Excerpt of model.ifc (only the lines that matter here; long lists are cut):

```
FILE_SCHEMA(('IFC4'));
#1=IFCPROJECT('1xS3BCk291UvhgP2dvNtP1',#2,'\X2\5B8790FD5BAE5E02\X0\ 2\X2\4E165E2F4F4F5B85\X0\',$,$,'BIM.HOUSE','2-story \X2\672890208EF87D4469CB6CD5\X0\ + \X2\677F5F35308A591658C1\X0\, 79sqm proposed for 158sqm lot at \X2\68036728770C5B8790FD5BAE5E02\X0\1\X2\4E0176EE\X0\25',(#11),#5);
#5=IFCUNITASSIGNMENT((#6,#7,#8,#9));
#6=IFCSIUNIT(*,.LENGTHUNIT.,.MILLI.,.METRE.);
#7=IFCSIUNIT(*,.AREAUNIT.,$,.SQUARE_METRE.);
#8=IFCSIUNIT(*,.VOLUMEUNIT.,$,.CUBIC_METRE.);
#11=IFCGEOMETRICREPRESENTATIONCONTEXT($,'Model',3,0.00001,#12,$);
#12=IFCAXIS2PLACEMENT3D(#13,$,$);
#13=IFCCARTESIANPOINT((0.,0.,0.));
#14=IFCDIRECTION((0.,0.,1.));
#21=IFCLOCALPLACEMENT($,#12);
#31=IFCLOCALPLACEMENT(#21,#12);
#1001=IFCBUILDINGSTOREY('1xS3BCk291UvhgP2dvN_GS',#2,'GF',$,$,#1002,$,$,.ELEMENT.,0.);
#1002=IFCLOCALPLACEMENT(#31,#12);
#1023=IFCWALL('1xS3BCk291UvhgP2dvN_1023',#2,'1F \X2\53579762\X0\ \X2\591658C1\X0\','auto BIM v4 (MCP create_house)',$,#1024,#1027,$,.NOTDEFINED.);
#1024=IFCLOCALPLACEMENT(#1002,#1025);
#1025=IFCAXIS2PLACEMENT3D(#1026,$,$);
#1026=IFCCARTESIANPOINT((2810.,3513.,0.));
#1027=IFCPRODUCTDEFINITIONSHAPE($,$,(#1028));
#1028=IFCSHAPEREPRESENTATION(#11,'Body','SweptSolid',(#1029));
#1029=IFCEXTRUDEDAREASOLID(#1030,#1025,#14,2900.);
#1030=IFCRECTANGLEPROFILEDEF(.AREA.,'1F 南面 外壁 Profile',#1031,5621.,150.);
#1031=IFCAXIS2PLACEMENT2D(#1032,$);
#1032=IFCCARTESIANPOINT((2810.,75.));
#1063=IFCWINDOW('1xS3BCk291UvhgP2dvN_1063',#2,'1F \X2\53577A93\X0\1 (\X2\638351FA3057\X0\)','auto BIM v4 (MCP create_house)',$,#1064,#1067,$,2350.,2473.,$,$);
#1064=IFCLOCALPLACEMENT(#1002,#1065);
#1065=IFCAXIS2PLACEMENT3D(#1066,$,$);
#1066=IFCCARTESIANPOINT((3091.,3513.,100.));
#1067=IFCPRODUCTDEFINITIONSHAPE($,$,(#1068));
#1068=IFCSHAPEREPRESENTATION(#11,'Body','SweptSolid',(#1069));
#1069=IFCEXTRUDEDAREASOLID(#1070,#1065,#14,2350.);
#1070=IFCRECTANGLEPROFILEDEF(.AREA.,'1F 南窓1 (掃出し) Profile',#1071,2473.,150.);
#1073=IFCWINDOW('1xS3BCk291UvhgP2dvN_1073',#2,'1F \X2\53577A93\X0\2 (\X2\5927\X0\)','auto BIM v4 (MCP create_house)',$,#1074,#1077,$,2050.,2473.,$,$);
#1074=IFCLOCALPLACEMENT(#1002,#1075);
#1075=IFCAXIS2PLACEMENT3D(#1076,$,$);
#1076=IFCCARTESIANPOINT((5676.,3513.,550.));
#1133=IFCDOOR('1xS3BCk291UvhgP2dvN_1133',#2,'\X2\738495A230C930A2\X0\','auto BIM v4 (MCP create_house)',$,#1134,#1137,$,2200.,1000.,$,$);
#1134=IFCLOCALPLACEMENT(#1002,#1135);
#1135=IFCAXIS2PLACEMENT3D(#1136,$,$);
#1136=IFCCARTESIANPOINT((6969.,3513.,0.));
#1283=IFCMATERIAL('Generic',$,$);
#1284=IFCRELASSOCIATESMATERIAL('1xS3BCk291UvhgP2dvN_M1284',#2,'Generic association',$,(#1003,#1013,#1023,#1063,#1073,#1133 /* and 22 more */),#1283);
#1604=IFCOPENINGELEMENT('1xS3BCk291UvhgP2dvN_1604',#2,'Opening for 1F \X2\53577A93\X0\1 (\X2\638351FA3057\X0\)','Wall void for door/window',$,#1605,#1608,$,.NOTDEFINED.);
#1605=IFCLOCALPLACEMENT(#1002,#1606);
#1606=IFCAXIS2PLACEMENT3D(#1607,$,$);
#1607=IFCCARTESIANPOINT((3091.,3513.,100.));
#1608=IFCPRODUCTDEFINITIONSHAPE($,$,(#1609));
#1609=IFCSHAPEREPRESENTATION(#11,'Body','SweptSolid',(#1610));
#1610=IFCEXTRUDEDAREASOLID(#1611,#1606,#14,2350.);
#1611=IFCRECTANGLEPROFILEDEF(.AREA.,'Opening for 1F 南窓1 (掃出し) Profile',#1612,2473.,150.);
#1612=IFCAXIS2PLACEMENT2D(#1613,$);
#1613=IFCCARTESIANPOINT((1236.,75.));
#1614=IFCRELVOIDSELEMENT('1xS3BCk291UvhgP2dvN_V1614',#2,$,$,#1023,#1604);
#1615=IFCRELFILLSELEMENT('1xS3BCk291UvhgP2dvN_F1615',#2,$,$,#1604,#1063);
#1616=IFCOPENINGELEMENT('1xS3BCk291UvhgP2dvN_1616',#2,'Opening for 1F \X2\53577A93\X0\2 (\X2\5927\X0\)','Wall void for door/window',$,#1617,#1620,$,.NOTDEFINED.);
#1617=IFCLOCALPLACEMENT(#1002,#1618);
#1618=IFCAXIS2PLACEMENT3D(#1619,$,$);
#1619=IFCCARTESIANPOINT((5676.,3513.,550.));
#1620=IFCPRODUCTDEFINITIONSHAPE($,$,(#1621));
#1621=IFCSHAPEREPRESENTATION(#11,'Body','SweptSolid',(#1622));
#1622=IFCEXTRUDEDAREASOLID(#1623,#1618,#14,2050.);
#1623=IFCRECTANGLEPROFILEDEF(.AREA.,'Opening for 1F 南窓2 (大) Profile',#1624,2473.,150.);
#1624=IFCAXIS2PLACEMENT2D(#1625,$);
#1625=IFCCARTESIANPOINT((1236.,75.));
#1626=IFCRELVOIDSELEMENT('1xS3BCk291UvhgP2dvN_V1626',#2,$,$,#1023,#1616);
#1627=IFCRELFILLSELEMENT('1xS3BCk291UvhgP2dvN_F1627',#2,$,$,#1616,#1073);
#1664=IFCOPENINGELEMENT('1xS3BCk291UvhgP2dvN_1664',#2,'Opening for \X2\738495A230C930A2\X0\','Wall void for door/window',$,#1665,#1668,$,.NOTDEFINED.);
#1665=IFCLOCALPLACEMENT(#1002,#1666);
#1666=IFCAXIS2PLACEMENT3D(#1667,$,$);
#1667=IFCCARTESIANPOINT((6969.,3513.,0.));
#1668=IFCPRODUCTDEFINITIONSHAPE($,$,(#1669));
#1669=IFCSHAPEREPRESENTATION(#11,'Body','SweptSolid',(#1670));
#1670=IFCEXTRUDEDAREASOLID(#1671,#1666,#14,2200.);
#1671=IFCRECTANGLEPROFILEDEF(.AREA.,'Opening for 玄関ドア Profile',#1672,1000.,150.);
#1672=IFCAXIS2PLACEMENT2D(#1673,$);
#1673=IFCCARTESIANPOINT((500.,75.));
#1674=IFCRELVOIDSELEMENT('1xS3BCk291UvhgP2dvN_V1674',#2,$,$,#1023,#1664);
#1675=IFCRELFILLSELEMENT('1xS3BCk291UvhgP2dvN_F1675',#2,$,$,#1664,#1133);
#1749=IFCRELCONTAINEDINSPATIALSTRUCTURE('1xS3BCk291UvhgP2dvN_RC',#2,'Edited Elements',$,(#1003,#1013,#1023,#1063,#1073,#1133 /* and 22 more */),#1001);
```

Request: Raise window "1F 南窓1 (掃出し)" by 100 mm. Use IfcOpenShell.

```python
import numpy as np
import ifcopenshell
import ifcopenshell.api.geometry
import ifcopenshell.util.placement
import ifcopenshell.util.unit

model = ifcopenshell.open("model.ifc")
unit_scale = ifcopenshell.util.unit.calculate_unit_scale(model)

window = model.by_guid("1xS3BCk291UvhgP2dvN_1063")
opening = window.FillsVoids[0].RelatingOpeningElement
dz = 0.1 / unit_scale

shift = np.array([0.0, 0.0, dz])
# The window is not placed relative to its opening, so move both.
for product in (opening, window):
    matrix = ifcopenshell.util.placement.get_local_placement(product.ObjectPlacement)
    matrix[:3, 3] += shift
    ifcopenshell.api.geometry.edit_object_placement(model, product=product, matrix=matrix, is_si=False)

print(f"moved by {dz * unit_scale:+.3f} m")

model.write("model-out.ifc")
```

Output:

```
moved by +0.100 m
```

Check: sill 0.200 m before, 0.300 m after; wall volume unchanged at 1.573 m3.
